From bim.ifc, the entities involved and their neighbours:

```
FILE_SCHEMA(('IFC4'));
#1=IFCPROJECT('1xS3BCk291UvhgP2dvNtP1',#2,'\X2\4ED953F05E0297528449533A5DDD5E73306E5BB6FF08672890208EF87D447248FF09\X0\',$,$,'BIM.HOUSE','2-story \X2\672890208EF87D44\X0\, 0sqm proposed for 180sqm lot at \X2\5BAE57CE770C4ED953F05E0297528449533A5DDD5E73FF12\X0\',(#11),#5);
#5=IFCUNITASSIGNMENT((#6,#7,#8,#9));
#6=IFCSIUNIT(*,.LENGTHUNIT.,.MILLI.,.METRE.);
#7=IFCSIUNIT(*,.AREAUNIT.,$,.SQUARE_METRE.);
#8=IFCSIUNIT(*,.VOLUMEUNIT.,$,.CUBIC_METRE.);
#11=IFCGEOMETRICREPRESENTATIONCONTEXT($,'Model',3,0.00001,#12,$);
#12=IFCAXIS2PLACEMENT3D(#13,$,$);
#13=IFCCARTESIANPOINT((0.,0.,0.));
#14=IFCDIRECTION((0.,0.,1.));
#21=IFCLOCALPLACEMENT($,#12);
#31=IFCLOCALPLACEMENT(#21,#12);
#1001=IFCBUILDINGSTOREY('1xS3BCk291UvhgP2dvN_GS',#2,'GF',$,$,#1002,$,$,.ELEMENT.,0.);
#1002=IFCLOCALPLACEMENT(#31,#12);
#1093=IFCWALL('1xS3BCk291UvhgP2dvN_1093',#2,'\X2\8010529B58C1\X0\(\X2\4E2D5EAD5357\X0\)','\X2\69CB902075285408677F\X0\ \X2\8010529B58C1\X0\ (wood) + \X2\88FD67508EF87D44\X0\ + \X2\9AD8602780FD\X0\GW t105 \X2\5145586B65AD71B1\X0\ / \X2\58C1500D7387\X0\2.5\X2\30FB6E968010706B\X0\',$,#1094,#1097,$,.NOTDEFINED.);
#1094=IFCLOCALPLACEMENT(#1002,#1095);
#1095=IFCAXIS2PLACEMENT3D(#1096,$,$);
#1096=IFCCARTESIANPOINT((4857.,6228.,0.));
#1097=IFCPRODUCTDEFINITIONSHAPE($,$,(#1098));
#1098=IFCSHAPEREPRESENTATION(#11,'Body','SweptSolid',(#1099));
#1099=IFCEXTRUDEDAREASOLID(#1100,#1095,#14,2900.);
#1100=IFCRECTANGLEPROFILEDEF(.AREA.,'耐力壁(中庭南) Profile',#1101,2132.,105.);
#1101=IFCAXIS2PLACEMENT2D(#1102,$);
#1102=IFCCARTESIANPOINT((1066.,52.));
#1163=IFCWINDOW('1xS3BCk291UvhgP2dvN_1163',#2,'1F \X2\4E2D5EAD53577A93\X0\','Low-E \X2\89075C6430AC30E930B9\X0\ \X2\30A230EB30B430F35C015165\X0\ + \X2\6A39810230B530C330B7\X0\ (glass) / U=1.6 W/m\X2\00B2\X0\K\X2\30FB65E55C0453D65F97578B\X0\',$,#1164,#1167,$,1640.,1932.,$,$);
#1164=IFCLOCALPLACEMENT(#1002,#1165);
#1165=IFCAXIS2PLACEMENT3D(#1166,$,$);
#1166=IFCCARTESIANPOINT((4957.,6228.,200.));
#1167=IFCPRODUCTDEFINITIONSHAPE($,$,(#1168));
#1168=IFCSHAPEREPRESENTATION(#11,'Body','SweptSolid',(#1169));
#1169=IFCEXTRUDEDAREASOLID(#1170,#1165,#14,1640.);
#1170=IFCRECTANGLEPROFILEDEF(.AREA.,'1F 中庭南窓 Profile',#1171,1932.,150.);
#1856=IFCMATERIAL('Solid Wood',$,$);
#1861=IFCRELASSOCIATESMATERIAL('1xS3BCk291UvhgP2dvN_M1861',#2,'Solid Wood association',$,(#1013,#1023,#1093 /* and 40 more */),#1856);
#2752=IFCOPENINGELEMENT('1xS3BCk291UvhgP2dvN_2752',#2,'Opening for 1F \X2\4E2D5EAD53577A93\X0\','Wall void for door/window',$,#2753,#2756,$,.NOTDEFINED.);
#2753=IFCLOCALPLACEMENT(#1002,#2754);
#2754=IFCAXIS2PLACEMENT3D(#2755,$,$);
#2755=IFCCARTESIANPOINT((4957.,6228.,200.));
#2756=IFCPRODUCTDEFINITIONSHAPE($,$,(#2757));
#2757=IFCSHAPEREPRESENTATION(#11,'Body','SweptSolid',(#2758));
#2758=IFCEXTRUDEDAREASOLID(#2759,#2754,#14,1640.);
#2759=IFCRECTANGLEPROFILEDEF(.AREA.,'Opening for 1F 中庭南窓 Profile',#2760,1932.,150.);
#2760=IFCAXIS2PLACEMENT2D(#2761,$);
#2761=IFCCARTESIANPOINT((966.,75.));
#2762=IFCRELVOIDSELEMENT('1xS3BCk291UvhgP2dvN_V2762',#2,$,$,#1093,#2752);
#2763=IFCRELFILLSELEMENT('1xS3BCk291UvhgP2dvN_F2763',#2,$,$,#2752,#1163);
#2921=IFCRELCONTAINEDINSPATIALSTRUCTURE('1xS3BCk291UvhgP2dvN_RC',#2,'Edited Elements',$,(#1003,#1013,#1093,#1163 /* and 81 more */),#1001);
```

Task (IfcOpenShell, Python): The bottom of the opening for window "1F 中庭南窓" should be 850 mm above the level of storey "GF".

```python
import numpy as np
import ifcopenshell
import ifcopenshell.api.geometry
import ifcopenshell.geom
import ifcopenshell.util.element
import ifcopenshell.util.placement
import ifcopenshell.util.shape
import ifcopenshell.util.unit

model = ifcopenshell.open("bim.ifc")
unit_scale = ifcopenshell.util.unit.calculate_unit_scale(model)

window = model.by_guid("1xS3BCk291UvhgP2dvN_1163")
opening = window.FillsVoids[0].RelatingOpeningElement
storey = ifcopenshell.util.element.get_container(window, ifc_class="IfcBuildingStorey")
level = ifcopenshell.util.placement.get_local_placement(storey.ObjectPlacement)[2, 3]

# The opening's origin need not be at the sill, so measure its lowest point.
shape = ifcopenshell.geom.create_shape(ifcopenshell.geom.settings(), opening)
bottom = ifcopenshell.util.shape.get_shape_bottom_elevation(shape, shape.geometry) / unit_scale
dz = level + 0.85 / unit_scale - bottom

shift = np.array([0.0, 0.0, dz])
# The window is not placed relative to its opening, so move both.
for product in (opening, window):
    matrix = ifcopenshell.util.placement.get_local_placement(product.ObjectPlacement)
    matrix[:3, 3] += shift
    ifcopenshell.api.geometry.edit_object_placement(model, product=product, matrix=matrix, is_si=False)

print(f"moved by {dz * unit_scale:+.3f} m")

model.write("bim_rev.ifc")
```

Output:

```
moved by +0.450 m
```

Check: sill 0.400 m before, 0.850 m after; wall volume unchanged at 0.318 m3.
